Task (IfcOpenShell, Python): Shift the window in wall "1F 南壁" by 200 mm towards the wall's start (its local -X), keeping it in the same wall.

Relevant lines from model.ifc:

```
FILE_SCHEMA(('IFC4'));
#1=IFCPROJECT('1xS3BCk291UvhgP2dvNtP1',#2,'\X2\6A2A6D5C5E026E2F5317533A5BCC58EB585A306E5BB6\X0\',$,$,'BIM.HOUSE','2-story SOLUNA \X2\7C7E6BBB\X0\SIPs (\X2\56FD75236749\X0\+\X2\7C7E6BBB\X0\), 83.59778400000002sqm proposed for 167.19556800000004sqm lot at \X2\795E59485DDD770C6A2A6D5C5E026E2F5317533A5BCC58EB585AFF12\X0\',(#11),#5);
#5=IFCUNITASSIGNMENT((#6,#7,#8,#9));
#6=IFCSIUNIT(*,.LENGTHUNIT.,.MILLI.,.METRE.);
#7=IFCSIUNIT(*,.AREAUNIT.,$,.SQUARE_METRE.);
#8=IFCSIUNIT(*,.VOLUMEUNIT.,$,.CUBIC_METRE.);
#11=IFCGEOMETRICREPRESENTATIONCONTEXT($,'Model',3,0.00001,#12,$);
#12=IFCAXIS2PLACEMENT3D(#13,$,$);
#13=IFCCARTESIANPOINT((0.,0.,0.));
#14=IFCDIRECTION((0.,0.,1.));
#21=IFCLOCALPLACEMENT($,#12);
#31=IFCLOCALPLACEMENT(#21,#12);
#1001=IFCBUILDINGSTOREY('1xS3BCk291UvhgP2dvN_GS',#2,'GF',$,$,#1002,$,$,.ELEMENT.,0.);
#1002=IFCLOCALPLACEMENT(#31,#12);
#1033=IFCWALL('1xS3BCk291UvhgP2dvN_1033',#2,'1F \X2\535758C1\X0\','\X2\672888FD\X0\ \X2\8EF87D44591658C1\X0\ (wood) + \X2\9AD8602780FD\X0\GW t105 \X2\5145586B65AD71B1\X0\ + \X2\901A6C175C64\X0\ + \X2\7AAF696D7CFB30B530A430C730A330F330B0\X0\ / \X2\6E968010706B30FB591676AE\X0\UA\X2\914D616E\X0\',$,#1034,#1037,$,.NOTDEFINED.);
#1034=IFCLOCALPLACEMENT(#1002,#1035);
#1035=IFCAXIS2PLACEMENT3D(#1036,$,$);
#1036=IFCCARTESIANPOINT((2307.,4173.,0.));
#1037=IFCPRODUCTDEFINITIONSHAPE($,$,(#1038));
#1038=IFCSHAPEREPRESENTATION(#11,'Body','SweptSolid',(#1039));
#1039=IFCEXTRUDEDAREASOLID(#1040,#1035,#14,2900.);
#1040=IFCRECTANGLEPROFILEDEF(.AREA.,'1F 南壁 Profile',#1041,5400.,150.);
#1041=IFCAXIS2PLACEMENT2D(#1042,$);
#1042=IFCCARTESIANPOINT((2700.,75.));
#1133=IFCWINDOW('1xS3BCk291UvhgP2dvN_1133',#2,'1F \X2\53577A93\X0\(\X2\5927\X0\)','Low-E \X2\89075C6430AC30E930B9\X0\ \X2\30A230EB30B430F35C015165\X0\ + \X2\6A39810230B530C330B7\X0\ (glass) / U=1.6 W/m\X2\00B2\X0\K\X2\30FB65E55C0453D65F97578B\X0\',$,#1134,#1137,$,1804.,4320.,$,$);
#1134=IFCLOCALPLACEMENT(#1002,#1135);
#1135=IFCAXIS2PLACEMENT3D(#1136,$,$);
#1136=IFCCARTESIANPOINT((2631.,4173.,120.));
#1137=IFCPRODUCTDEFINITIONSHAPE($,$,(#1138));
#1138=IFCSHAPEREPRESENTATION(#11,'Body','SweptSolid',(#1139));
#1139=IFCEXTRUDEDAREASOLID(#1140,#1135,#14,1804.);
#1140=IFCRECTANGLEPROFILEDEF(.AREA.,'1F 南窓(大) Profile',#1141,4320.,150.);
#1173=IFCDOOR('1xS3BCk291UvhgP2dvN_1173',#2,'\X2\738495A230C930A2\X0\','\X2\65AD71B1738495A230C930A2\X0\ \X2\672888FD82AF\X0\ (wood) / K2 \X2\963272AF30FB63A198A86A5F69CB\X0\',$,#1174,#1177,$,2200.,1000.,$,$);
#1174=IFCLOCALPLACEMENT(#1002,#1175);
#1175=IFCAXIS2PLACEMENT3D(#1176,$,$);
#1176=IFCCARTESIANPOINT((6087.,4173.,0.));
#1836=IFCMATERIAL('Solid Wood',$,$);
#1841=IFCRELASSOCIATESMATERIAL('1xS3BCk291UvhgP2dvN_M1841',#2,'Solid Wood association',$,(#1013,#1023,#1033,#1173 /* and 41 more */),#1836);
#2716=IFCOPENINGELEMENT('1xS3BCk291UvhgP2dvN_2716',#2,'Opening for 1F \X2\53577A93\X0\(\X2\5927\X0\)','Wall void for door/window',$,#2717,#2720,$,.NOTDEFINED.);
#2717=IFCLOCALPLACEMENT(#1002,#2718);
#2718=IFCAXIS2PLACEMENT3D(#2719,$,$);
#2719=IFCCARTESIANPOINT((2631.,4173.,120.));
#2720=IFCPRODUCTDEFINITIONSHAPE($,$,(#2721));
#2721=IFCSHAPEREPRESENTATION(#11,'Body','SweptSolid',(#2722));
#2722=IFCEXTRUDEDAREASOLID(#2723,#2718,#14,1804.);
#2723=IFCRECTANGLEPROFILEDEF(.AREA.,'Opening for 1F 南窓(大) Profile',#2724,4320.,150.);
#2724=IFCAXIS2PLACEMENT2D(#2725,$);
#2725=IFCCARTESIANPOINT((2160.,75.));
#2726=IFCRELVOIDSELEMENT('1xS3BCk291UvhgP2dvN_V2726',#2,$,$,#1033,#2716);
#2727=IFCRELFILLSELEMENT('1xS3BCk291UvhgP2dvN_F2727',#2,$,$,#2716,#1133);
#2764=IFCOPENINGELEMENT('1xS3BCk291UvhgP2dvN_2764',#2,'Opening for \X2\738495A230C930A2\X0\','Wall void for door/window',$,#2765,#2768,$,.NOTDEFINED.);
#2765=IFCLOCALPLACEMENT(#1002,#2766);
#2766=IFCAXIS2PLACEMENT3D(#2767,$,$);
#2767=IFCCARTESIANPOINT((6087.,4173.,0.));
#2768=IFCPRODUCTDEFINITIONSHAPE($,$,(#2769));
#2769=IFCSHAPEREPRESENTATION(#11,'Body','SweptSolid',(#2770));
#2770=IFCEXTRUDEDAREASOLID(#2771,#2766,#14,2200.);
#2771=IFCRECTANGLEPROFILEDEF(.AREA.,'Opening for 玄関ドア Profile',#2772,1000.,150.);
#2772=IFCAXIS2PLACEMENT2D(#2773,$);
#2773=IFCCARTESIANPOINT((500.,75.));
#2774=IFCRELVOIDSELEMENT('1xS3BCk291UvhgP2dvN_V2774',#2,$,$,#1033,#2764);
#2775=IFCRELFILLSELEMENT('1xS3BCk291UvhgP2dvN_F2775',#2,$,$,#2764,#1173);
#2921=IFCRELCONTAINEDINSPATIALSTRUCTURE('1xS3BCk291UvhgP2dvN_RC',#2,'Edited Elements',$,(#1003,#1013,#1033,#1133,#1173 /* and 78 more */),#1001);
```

```python
import ifcopenshell
import ifcopenshell.api.geometry
import ifcopenshell.util.placement

model = ifcopenshell.open("model.ifc")

window = model.by_guid("1xS3BCk291UvhgP2dvN_1133")
opening = window.FillsVoids[0].RelatingOpeningElement
wall = opening.VoidsElements[0].RelatingBuildingElement

wall_matrix = ifcopenshell.util.placement.get_local_placement(wall.ObjectPlacement)
shift = wall_matrix[:3, 0] * -200.0
before = ifcopenshell.util.placement.get_local_placement(window.ObjectPlacement)[:3, 3].copy()

# The window is not placed relative to its opening, so move both.
for product in (opening, window):
    matrix = ifcopenshell.util.placement.get_local_placement(product.ObjectPlacement)
    matrix[:3, 3] += shift
    ifcopenshell.api.geometry.edit_object_placement(model, product=product, matrix=matrix, is_si=False)

after = ifcopenshell.util.placement.get_local_placement(window.ObjectPlacement)[:3, 3]
print("window moved by", (after - before).round(3) + 0.0)

model.write("model-out.ifc")
```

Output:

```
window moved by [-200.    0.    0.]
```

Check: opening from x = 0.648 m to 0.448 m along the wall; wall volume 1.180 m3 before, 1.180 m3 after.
